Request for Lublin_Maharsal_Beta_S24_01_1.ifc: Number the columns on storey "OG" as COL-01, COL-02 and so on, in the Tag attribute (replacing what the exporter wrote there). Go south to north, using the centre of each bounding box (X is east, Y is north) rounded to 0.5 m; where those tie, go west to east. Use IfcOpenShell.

First a look at what the model holds.

```python
import ifcopenshell
import ifcopenshell.util.element
import ifcopenshell.util.placement

model = ifcopenshell.open("Lublin_Maharsal_Beta_S24_01_1.ifc")
print(model.schema)
storey = next(s for s in model.by_type("IfcBuildingStorey") if s.Name == "OG")
columns = [e for e in ifcopenshell.util.element.get_decomposition(storey) if e.is_a("IfcColumn")]
for e in sorted(columns, key=lambda e: e.id()):
    origin = ifcopenshell.util.placement.get_local_placement(e.ObjectPlacement)[:3, 3]
    print(e.id(), e.Tag, e.Name, origin.round(2) + 0.0, sep=" | ")
```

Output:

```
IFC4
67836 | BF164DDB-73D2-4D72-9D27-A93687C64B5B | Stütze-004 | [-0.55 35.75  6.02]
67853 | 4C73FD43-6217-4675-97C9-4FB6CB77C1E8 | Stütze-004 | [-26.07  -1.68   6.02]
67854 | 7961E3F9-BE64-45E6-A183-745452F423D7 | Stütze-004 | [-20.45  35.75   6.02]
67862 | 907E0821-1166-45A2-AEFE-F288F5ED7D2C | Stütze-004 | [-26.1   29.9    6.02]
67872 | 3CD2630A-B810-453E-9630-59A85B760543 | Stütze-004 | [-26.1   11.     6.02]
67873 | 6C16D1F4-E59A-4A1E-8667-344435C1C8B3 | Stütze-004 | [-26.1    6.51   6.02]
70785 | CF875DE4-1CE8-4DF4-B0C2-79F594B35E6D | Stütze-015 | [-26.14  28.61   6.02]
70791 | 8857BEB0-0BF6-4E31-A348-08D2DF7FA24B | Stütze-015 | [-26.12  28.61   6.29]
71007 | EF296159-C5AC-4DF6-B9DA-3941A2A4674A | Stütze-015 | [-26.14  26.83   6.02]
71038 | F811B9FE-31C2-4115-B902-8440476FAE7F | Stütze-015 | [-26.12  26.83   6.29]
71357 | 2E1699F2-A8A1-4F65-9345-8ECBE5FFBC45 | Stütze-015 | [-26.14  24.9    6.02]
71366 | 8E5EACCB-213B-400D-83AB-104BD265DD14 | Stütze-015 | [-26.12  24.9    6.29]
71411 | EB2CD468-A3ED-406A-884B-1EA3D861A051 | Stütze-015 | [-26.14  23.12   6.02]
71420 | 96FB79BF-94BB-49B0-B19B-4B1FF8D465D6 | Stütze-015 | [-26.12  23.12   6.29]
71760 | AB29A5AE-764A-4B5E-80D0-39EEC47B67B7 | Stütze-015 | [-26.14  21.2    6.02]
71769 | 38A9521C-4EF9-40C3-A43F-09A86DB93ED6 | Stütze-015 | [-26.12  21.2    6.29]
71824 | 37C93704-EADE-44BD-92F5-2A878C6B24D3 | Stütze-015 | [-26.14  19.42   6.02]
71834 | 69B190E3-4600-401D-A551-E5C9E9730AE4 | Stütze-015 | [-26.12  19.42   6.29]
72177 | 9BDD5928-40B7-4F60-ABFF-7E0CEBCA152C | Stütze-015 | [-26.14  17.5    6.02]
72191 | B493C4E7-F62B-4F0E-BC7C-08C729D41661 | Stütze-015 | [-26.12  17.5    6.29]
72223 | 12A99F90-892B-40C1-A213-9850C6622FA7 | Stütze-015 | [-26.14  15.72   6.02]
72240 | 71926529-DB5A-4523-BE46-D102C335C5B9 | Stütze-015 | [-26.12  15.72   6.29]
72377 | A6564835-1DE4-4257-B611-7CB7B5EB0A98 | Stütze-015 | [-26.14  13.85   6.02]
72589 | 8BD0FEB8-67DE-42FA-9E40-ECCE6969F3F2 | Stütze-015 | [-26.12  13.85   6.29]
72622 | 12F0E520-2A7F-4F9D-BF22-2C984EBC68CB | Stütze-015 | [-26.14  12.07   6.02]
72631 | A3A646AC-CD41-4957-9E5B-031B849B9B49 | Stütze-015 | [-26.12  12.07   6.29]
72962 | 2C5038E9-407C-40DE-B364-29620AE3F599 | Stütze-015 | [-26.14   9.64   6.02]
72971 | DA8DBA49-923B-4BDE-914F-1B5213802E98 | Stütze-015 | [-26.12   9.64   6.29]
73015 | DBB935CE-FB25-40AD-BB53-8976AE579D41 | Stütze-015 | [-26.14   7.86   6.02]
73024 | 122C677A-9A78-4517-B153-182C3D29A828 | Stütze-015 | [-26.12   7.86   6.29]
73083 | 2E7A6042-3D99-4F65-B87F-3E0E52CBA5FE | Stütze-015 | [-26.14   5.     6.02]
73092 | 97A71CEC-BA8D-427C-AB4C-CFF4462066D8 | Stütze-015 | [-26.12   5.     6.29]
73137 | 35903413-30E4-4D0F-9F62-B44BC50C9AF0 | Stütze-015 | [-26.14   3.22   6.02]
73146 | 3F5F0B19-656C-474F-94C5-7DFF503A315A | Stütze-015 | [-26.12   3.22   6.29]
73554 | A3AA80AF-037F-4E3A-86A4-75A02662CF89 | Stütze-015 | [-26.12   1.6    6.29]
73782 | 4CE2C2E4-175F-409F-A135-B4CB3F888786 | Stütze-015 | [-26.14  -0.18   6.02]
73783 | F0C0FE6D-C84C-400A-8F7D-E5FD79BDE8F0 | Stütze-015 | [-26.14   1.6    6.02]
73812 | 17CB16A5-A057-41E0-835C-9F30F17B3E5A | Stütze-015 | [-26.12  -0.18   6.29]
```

```python
import ifcopenshell
import ifcopenshell.geom
import ifcopenshell.util.element
import ifcopenshell.util.shape

model = ifcopenshell.open("Lublin_Maharsal_Beta_S24_01_1.ifc")
settings = ifcopenshell.geom.settings()
settings.set("use-world-coords", True)


def centre(element):
    shape = ifcopenshell.geom.create_shape(settings, element)
    return ifcopenshell.util.shape.get_bbox_centroid(shape.geometry)


storey = next(s for s in model.by_type("IfcBuildingStorey") if s.Name == "OG")
columns = [e for e in ifcopenshell.util.element.get_decomposition(storey) if e.is_a("IfcColumn")]

# Insertion points can sit at a corner or the storey origin, so sort by the geometry (in metres).
centres = {e: centre(e) for e in columns}
columns.sort(key=lambda e: (round(centres[e][1] / 0.5), centres[e][0]))

for i, e in enumerate(columns, start=1):
    number = f"COL-{i:02d}"
    e.Tag = number
    print(e.id(), number)

model.write("Lublin_Maharsal_Beta_S24_01_1-out.ifc")
```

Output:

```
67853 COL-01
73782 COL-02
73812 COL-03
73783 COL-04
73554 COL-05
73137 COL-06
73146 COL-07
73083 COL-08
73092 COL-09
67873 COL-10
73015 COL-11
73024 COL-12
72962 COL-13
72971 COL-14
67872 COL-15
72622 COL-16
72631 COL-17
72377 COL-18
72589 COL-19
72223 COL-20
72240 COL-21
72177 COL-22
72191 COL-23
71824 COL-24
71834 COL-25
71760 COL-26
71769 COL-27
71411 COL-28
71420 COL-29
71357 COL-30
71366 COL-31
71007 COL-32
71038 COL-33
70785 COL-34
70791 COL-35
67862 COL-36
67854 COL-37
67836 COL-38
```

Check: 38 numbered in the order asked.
